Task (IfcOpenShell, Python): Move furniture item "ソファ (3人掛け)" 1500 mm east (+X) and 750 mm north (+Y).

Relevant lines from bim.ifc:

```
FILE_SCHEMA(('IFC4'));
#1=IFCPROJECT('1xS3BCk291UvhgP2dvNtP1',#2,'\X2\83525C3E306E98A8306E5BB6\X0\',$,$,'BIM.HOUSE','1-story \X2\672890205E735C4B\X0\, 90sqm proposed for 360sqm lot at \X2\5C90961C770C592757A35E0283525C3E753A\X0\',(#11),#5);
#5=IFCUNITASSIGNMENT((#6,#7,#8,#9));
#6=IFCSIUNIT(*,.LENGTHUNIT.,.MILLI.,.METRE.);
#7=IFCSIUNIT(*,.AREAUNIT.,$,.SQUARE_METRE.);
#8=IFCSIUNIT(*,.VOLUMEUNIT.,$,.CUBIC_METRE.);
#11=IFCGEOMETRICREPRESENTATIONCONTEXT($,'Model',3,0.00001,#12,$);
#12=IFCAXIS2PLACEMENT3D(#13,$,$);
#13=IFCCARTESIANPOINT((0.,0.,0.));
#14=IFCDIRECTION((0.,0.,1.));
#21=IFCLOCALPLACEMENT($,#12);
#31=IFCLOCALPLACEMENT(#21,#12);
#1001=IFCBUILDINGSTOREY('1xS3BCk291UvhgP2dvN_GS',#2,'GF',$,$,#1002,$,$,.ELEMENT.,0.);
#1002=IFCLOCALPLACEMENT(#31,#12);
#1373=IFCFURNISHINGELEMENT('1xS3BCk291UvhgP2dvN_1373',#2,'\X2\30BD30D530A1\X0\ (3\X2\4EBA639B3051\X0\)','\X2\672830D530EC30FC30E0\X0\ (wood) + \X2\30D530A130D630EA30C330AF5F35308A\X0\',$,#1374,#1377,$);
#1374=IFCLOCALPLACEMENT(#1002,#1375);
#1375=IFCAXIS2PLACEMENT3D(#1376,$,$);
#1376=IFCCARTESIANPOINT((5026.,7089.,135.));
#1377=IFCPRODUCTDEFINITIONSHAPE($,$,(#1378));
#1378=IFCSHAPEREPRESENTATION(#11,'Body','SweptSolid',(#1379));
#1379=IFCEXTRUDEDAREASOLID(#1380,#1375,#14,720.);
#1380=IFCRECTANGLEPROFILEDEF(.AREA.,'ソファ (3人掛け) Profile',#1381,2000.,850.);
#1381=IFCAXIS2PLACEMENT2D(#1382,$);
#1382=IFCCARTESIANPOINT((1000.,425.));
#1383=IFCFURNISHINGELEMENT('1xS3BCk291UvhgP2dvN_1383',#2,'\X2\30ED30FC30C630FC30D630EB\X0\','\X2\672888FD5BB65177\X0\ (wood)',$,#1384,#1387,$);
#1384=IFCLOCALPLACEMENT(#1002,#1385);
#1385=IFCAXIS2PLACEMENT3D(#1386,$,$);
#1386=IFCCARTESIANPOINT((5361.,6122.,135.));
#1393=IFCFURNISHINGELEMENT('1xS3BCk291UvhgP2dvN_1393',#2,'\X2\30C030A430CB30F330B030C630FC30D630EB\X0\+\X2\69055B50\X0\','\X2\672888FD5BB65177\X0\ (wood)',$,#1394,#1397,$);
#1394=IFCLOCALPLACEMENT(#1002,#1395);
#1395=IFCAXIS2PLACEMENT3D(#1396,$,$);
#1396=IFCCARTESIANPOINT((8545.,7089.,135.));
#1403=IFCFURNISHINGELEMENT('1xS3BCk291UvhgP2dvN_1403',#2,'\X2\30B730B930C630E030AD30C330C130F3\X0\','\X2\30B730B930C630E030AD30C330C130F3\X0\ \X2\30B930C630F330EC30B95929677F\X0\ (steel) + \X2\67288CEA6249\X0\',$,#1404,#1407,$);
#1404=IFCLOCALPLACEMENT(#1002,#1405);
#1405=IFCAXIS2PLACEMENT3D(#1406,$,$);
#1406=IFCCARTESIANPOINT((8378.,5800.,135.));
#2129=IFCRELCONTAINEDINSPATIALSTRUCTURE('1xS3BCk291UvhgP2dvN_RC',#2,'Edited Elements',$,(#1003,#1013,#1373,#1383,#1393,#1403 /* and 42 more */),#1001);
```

```python
import ifcopenshell
import ifcopenshell.api.geometry
import ifcopenshell.util.placement
import ifcopenshell.util.unit

model = ifcopenshell.open("bim.ifc")
unit_scale = ifcopenshell.util.unit.calculate_unit_scale(model)

item = model.by_guid("1xS3BCk291UvhgP2dvN_1373")
matrix = ifcopenshell.util.placement.get_local_placement(item.ObjectPlacement)
matrix[0, 3] += 1.5 / unit_scale
matrix[1, 3] += 0.75 / unit_scale
ifcopenshell.api.geometry.edit_object_placement(model, product=item, matrix=matrix, is_si=False)

print(ifcopenshell.util.placement.get_local_placement(item.ObjectPlacement).round(3) + 0.0)

model.write("bim_rev.ifc")
```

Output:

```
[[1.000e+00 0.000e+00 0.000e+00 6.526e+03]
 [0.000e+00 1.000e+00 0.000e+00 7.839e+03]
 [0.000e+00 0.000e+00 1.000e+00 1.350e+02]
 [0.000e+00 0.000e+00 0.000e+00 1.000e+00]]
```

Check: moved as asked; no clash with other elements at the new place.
